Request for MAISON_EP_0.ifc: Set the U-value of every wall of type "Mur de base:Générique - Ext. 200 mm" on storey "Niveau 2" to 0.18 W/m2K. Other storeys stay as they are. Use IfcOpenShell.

First a look at what the model holds.

```python
import ifcopenshell
import ifcopenshell.util.element

model = ifcopenshell.open("MAISON_EP_0.ifc")
print(model.schema)
storey = next(s for s in model.by_type("IfcBuildingStorey") if s.Name == "Niveau 2")
walls = [e for e in ifcopenshell.util.element.get_decomposition(storey) if e.is_a("IfcWall")]
seen = {}
for e in walls:
    element_type = ifcopenshell.util.element.get_type(e)
    key = (element_type.Name if element_type != e and element_type else None, ifcopenshell.util.element.get_pset(e, "Pset_WallCommon", "ThermalTransmittance"))
    seen[key] = seen.get(key, 0) + 1
for (name, value), count in sorted(seen.items(), key=str):
    print(count, "x", name, "|", value)
```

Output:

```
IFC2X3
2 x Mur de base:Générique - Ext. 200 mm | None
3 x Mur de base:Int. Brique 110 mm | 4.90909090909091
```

```python
import ifcopenshell
import ifcopenshell.api.pset
import ifcopenshell.util.element

model = ifcopenshell.open("MAISON_EP_0.ifc")

storey = next(s for s in model.by_type("IfcBuildingStorey") if s.Name == "Niveau 2")
walls = [e for e in ifcopenshell.util.element.get_decomposition(storey) if e.is_a("IfcWall")]

count = 0
for e in walls:
    element_type = ifcopenshell.util.element.get_type(e)
    if element_type in (None, e) or element_type.Name != "Mur de base:Générique - Ext. 200 mm":
        continue
    found = ifcopenshell.util.element.get_pset(e, "Pset_WallCommon", should_inherit=False)
    if found:
        pset = model.by_id(found["id"])
        if len(ifcopenshell.util.element.get_elements_by_pset(pset)) > 1:
            pset = ifcopenshell.api.pset.unshare_pset(model, products=[e], pset=pset)[0]
    else:
        pset = ifcopenshell.api.pset.add_pset(model, product=e, name="Pset_WallCommon")
    ifcopenshell.api.pset.edit_pset(model, pset=pset, properties={"ThermalTransmittance": 0.18})
    count += 1

print(count, "walls updated")

model.write("MAISON_EP_0-out.ifc")
```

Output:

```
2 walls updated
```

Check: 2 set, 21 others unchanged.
